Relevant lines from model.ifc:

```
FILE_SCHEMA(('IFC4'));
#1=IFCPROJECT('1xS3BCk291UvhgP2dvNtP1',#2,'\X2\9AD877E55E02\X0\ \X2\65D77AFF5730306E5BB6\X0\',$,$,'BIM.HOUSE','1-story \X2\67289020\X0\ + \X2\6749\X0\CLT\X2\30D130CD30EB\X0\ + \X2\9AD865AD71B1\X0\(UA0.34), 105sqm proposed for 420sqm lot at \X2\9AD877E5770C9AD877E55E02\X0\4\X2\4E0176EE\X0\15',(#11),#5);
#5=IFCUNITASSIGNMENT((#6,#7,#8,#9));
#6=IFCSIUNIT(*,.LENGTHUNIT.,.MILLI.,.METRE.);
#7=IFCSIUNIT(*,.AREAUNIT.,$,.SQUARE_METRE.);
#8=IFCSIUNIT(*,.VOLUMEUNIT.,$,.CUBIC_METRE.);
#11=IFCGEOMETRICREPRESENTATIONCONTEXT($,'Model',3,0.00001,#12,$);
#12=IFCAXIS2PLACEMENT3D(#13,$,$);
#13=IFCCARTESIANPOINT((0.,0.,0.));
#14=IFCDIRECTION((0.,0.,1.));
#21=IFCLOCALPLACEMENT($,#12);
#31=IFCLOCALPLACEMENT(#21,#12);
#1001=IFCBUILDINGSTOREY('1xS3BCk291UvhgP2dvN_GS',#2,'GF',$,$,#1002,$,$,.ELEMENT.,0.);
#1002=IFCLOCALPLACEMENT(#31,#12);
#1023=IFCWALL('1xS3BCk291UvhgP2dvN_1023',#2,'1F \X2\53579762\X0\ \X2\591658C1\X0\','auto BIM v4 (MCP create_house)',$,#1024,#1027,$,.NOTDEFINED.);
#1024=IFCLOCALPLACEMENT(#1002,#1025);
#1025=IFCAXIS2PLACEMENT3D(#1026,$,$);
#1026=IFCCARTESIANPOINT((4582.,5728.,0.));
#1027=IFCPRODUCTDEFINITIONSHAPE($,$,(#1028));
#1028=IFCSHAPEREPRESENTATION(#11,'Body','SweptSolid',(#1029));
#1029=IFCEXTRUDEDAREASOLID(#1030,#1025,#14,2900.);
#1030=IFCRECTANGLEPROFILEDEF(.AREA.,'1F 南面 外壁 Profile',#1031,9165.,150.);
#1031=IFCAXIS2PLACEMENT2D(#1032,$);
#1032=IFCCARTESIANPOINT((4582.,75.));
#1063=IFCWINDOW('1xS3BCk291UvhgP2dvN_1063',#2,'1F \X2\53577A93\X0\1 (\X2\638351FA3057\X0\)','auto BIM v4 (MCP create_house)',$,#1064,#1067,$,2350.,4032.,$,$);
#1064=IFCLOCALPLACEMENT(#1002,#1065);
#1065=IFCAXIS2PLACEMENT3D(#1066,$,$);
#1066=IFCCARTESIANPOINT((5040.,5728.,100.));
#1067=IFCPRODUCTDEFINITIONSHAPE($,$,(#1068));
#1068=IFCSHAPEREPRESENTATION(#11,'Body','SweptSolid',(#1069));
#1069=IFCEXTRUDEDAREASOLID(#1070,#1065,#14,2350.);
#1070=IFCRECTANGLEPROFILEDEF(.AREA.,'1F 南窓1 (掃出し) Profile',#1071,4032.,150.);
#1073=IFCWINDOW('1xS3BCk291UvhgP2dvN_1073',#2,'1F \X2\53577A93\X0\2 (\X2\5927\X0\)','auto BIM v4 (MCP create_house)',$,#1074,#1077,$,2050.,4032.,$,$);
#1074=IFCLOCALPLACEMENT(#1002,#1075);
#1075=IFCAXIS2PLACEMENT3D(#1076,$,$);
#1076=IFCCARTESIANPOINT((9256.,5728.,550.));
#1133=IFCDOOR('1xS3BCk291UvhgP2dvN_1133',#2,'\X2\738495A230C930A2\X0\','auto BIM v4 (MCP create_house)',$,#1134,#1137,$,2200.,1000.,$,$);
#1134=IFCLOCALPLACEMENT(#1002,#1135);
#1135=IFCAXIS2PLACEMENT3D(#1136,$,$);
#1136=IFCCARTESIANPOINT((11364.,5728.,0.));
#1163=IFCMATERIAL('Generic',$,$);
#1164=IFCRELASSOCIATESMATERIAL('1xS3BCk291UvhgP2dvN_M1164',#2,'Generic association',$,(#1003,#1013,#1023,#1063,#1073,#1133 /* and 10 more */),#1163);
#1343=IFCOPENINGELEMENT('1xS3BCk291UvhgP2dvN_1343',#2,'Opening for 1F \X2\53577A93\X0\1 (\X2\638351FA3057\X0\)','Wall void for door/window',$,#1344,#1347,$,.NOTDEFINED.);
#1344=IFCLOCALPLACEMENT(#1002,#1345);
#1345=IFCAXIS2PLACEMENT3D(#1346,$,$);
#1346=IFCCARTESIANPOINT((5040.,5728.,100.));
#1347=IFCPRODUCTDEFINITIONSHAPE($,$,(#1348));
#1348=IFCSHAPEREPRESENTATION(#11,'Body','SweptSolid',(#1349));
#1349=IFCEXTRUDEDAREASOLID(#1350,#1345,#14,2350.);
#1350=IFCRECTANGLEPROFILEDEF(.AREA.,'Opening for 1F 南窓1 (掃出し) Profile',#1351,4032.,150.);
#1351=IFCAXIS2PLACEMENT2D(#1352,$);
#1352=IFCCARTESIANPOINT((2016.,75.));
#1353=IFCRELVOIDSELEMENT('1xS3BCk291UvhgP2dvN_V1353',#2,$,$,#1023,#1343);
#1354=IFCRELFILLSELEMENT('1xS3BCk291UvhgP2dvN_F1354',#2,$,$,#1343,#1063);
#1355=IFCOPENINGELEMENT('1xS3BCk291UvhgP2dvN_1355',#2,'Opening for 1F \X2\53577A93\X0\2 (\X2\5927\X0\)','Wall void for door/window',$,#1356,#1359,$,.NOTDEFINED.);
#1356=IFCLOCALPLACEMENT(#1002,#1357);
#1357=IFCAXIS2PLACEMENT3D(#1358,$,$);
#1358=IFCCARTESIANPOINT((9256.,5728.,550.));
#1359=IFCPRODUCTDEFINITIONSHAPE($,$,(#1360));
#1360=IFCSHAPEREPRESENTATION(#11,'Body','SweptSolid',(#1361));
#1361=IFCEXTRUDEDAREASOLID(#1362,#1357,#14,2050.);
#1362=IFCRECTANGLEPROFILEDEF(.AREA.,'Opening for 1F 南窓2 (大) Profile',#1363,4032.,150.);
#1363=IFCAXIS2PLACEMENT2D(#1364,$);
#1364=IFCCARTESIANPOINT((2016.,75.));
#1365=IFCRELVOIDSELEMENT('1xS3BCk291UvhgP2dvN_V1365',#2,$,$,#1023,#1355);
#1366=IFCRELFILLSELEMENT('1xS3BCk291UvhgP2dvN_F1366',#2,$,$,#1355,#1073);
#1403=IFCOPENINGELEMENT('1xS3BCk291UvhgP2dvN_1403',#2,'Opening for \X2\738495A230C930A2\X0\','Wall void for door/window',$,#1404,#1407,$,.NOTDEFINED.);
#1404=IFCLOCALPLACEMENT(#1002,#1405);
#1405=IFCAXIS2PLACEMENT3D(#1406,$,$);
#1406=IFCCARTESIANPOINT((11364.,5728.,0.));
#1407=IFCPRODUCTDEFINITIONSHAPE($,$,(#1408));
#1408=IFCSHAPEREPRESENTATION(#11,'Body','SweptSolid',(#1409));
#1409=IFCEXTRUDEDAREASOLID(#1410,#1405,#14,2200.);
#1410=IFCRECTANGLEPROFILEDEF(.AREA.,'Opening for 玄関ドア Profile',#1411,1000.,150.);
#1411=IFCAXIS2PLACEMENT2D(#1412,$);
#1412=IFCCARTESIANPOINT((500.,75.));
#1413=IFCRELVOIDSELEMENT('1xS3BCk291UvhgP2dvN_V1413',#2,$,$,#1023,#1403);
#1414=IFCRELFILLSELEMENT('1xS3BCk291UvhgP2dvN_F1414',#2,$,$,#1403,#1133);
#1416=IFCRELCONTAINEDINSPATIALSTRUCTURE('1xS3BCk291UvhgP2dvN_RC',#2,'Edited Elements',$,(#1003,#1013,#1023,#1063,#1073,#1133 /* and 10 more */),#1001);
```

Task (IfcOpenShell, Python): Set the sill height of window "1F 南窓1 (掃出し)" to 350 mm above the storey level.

```python
import numpy as np
import ifcopenshell
import ifcopenshell.api.geometry
import ifcopenshell.geom
import ifcopenshell.util.element
import ifcopenshell.util.placement
import ifcopenshell.util.shape
import ifcopenshell.util.unit

model = ifcopenshell.open("model.ifc")
unit_scale = ifcopenshell.util.unit.calculate_unit_scale(model)

window = model.by_guid("1xS3BCk291UvhgP2dvN_1063")
opening = window.FillsVoids[0].RelatingOpeningElement
storey = ifcopenshell.util.element.get_container(window, ifc_class="IfcBuildingStorey")
level = ifcopenshell.util.placement.get_local_placement(storey.ObjectPlacement)[2, 3]

# The opening's origin need not be at the sill, so measure its lowest point.
shape = ifcopenshell.geom.create_shape(ifcopenshell.geom.settings(), opening)
bottom = ifcopenshell.util.shape.get_shape_bottom_elevation(shape, shape.geometry) / unit_scale
dz = level + 0.35 / unit_scale - bottom

shift = np.array([0.0, 0.0, dz])
# The window is not placed relative to its opening, so move both.
for product in (opening, window):
    matrix = ifcopenshell.util.placement.get_local_placement(product.ObjectPlacement)
    matrix[:3, 3] += shift
    ifcopenshell.api.geometry.edit_object_placement(model, product=product, matrix=matrix, is_si=False)

print(f"moved by {dz * unit_scale:+.3f} m")

model.write("model-out.ifc")
```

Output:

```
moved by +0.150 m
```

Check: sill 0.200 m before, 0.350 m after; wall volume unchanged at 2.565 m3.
